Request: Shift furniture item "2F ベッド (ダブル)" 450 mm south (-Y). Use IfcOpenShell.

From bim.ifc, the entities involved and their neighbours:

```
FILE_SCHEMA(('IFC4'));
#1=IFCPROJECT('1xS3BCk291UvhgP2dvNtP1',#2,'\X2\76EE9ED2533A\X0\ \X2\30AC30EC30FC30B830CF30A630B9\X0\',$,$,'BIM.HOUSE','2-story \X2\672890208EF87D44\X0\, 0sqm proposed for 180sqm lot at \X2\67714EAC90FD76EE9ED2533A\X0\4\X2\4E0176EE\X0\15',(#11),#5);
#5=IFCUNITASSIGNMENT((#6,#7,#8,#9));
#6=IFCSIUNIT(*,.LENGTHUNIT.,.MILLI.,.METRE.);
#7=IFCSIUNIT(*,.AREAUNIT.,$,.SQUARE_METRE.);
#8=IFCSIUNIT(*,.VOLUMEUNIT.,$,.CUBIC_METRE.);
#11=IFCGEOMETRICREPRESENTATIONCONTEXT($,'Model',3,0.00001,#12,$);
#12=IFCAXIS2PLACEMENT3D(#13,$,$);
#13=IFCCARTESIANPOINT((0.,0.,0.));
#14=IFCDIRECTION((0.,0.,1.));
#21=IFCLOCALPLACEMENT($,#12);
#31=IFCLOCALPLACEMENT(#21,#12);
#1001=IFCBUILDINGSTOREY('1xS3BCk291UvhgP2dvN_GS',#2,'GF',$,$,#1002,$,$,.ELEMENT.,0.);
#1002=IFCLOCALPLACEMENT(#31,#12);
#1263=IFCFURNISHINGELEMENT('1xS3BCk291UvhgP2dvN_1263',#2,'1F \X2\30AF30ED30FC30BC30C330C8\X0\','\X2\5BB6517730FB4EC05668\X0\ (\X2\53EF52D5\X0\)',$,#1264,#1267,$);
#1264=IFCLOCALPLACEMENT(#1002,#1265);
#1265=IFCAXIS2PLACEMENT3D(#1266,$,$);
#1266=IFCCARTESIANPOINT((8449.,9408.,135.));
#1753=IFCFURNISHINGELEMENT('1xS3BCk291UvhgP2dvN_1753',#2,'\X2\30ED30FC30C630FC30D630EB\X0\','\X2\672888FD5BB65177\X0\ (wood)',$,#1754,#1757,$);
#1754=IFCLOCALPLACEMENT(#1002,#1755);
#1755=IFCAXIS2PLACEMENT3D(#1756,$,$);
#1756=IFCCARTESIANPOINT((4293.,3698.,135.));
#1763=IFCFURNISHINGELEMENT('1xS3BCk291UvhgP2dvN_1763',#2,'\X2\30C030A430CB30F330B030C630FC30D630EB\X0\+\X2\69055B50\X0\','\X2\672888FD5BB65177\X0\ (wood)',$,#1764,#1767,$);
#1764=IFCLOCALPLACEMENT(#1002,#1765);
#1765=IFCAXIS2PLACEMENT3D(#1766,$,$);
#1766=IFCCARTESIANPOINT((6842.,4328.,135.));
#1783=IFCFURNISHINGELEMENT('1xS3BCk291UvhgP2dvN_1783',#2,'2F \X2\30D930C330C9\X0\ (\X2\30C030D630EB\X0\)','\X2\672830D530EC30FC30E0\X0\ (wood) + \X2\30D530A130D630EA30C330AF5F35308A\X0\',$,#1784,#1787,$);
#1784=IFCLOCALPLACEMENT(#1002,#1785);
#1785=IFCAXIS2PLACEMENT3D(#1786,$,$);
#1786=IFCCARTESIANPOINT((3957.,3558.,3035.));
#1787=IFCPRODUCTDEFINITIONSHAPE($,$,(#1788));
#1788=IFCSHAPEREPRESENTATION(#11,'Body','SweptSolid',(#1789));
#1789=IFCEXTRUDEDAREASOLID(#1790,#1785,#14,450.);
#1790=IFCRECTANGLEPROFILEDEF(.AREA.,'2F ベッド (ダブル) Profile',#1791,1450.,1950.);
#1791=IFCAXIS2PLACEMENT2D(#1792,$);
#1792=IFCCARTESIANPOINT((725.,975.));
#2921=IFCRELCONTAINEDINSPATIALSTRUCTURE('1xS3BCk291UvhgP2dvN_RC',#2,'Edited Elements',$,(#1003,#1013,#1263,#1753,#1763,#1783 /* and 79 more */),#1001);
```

```python
import ifcopenshell
import ifcopenshell.api.geometry
import ifcopenshell.util.placement

model = ifcopenshell.open("bim.ifc")

item = model.by_id(1783)
matrix = ifcopenshell.util.placement.get_local_placement(item.ObjectPlacement)
matrix[1, 3] -= 450.0
ifcopenshell.api.geometry.edit_object_placement(model, product=item, matrix=matrix, is_si=False)

print(ifcopenshell.util.placement.get_local_placement(item.ObjectPlacement).round(3) + 0.0)

model.write("bim_rev.ifc")
```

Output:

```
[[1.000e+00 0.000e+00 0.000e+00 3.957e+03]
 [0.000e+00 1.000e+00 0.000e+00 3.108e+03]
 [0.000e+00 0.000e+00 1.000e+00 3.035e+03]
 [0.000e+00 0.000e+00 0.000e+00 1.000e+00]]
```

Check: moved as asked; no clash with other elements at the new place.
